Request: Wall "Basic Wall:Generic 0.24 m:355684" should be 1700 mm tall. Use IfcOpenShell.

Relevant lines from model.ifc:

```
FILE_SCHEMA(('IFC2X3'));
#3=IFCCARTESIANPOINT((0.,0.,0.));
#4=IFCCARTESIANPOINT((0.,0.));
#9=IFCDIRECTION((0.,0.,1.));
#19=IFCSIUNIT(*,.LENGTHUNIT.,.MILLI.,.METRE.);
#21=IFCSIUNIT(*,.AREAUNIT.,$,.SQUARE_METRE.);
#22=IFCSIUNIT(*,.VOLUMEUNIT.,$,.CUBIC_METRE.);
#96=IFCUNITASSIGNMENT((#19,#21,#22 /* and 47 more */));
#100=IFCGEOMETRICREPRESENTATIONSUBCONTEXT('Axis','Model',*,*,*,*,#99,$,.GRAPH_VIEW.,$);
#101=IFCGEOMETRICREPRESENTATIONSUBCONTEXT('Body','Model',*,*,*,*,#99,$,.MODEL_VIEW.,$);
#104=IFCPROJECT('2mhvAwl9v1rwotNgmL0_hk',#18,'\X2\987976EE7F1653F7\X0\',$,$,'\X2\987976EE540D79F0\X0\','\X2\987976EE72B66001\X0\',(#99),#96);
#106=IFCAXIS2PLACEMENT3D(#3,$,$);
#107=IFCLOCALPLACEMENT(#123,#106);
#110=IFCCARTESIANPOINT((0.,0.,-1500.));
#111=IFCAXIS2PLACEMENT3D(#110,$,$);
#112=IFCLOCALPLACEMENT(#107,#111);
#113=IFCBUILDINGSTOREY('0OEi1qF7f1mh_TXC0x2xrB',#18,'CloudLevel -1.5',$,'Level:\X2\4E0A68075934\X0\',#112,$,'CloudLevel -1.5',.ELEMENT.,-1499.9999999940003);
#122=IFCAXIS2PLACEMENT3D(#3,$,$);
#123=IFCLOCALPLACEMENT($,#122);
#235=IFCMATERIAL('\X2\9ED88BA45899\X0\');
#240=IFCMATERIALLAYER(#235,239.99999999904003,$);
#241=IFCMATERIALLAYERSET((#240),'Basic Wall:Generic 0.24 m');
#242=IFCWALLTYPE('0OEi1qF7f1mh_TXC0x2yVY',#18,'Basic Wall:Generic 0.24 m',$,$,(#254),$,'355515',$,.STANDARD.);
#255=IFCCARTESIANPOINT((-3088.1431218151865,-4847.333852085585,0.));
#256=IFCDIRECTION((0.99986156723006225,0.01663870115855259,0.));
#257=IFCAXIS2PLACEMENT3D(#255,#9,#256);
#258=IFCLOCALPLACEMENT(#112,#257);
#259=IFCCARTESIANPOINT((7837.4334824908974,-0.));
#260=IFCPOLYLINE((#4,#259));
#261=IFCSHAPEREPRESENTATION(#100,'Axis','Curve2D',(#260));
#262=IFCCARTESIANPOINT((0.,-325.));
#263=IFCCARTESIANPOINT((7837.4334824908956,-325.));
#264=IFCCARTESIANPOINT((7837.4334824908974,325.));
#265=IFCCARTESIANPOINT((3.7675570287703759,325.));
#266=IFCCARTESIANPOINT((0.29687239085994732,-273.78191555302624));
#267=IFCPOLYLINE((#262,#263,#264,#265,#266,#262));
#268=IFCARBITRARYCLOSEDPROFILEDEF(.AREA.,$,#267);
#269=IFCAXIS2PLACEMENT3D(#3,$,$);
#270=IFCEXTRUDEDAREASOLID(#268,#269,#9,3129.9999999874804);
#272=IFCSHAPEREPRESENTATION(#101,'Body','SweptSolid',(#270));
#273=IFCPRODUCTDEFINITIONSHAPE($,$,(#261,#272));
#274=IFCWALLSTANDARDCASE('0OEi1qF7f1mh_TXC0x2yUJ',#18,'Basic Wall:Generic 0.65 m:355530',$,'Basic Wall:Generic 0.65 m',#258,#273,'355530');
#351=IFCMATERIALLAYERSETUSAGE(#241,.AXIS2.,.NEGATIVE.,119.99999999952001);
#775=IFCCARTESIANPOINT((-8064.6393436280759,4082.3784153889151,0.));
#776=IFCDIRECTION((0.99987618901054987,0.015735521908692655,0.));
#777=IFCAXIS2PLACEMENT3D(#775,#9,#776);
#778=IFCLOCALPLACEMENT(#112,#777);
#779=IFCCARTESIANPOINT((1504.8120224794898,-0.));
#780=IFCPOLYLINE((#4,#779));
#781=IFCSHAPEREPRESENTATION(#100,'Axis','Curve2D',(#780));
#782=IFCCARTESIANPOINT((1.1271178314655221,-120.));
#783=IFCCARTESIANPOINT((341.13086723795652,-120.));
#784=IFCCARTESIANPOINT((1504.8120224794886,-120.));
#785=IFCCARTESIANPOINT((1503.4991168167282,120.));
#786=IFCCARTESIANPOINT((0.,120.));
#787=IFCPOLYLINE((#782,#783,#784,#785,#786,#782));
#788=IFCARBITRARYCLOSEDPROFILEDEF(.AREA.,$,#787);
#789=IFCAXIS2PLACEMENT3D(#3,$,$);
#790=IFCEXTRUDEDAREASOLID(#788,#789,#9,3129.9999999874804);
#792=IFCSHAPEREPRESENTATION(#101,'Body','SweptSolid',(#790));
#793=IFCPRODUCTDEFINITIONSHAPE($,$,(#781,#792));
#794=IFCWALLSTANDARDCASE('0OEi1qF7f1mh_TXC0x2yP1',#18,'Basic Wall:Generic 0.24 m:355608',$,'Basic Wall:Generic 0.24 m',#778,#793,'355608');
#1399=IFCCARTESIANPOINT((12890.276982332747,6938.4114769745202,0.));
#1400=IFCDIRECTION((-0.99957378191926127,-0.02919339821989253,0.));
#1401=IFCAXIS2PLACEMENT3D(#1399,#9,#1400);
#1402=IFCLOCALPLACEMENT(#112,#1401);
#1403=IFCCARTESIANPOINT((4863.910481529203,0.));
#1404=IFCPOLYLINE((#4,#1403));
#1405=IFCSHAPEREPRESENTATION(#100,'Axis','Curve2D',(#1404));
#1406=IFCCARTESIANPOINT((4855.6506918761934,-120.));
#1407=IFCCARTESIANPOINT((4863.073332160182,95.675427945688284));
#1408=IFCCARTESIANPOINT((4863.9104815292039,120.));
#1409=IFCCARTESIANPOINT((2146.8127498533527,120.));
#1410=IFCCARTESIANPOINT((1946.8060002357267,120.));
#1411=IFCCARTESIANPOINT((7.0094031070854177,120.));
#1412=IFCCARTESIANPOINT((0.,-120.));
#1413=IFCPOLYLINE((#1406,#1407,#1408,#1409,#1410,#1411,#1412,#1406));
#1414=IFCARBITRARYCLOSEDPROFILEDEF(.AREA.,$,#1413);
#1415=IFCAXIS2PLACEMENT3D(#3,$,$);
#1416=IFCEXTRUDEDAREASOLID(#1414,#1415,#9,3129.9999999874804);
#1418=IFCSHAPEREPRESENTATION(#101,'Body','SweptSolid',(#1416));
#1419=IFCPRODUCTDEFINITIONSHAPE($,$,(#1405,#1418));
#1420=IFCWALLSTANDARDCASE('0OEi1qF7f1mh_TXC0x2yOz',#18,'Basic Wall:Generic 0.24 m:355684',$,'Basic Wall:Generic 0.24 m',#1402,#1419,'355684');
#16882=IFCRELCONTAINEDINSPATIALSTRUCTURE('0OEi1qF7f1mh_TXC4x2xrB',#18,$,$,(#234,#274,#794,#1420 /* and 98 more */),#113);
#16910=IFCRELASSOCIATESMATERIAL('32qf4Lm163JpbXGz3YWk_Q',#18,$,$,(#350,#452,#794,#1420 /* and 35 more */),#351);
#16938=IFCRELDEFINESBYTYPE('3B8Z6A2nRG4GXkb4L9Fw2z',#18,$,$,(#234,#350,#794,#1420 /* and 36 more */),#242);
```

```python
import ifcopenshell
import ifcopenshell.geom
import ifcopenshell.util.representation
import ifcopenshell.util.shape
import ifcopenshell.util.unit

model = ifcopenshell.open("model.ifc")
unit_scale = ifcopenshell.util.unit.calculate_unit_scale(model)
settings = ifcopenshell.geom.settings()


def volume(element):
    """Net volume in cubic metres, openings subtracted."""
    shape = ifcopenshell.geom.create_shape(settings, element)
    return ifcopenshell.util.shape.get_volume(shape.geometry)


wall = model.by_id(1420)
before = volume(wall)

body = ifcopenshell.util.representation.get_representation(wall, "Model", "Body")
solid = body.Items[0]
old_height = solid.Depth
solid.Depth = 1.7 / unit_scale
after = volume(wall)

print(f"height {old_height:g} -> {solid.Depth:g}, volume {before:.3f} -> {after:.3f} m3")

model.write("model_v2.ifc")
```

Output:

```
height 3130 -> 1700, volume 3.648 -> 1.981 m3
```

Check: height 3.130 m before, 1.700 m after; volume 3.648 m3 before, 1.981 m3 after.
